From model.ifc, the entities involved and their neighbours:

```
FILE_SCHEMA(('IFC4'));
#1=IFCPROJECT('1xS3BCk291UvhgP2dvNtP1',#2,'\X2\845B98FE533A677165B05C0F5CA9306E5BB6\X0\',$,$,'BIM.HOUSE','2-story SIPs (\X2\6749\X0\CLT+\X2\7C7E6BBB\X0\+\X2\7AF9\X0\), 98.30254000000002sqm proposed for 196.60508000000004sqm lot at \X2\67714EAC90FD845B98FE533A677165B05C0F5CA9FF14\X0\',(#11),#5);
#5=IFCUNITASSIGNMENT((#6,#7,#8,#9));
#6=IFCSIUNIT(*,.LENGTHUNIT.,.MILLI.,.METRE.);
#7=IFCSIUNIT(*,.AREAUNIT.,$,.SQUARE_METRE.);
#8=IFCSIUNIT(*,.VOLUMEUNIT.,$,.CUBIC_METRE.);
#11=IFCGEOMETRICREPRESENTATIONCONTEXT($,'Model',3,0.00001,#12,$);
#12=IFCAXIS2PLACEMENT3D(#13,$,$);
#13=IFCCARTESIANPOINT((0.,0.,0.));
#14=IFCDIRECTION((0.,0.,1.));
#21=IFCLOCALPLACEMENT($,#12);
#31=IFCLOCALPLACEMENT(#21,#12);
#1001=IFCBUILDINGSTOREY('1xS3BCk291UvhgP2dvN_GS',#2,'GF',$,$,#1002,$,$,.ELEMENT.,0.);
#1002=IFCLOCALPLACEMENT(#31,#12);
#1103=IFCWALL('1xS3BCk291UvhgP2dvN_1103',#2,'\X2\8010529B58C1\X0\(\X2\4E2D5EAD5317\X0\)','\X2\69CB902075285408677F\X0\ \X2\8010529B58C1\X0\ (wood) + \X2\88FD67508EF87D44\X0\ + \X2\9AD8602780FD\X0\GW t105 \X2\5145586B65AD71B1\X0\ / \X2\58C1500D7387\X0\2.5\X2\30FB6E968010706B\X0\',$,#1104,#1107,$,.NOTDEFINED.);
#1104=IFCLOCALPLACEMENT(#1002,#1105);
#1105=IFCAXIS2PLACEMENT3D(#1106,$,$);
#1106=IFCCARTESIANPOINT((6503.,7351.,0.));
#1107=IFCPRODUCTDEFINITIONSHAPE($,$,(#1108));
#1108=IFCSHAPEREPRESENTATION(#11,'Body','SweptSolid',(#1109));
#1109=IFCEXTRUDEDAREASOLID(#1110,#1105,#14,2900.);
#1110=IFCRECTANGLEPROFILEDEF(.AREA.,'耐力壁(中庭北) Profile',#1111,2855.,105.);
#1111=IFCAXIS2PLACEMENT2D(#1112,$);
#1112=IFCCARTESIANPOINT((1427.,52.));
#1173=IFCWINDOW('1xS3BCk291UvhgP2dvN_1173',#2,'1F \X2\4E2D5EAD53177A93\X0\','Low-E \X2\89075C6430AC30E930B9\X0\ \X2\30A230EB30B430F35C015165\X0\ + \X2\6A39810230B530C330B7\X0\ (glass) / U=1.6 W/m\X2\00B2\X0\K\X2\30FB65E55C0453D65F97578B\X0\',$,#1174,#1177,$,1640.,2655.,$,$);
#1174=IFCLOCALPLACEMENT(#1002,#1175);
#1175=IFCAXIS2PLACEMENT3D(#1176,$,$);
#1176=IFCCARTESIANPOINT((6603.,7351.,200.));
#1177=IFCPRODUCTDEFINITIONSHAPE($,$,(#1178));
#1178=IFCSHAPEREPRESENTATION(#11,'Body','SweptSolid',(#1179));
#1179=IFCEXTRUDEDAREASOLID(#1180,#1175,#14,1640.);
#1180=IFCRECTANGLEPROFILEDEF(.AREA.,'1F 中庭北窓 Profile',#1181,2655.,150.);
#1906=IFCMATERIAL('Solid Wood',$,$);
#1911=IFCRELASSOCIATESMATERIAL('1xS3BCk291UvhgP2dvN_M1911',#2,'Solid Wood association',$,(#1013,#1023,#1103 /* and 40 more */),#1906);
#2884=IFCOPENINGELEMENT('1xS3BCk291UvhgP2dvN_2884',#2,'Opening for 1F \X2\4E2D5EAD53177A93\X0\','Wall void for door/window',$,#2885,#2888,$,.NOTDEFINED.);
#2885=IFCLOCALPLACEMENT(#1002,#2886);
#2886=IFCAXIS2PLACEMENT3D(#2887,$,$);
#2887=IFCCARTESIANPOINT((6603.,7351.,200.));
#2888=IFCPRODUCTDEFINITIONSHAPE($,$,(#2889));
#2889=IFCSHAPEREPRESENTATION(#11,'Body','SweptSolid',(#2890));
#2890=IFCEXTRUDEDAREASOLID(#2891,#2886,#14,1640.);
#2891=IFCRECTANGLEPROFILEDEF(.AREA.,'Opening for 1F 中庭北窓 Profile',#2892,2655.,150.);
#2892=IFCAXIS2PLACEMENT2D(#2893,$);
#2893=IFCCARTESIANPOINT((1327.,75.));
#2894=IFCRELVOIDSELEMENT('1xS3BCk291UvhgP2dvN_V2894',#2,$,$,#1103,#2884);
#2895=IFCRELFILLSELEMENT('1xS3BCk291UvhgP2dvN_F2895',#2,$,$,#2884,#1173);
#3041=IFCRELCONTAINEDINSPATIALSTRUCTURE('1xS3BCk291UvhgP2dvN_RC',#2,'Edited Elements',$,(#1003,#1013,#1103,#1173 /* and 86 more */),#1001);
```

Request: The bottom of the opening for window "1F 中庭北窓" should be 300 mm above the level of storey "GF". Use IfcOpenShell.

```python
import numpy as np
import ifcopenshell
import ifcopenshell.api.geometry
import ifcopenshell.geom
import ifcopenshell.util.element
import ifcopenshell.util.placement
import ifcopenshell.util.shape
import ifcopenshell.util.unit

model = ifcopenshell.open("model.ifc")
unit_scale = ifcopenshell.util.unit.calculate_unit_scale(model)

window = model.by_guid("1xS3BCk291UvhgP2dvN_1173")
opening = window.FillsVoids[0].RelatingOpeningElement
storey = ifcopenshell.util.element.get_container(window, ifc_class="IfcBuildingStorey")
level = ifcopenshell.util.placement.get_local_placement(storey.ObjectPlacement)[2, 3]

# The opening's origin need not be at the sill, so measure its lowest point.
shape = ifcopenshell.geom.create_shape(ifcopenshell.geom.settings(), opening)
bottom = ifcopenshell.util.shape.get_shape_bottom_elevation(shape, shape.geometry) / unit_scale
dz = level + 300.0 - bottom

shift = np.array([0.0, 0.0, dz])
# The window is not placed relative to its opening, so move both.
for product in (opening, window):
    matrix = ifcopenshell.util.placement.get_local_placement(product.ObjectPlacement)
    matrix[:3, 3] += shift
    ifcopenshell.api.geometry.edit_object_placement(model, product=product, matrix=matrix, is_si=False)

print(f"moved by {dz * unit_scale:+.3f} m")

model.write("model-out.ifc")
```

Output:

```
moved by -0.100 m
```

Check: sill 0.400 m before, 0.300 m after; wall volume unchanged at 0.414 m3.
